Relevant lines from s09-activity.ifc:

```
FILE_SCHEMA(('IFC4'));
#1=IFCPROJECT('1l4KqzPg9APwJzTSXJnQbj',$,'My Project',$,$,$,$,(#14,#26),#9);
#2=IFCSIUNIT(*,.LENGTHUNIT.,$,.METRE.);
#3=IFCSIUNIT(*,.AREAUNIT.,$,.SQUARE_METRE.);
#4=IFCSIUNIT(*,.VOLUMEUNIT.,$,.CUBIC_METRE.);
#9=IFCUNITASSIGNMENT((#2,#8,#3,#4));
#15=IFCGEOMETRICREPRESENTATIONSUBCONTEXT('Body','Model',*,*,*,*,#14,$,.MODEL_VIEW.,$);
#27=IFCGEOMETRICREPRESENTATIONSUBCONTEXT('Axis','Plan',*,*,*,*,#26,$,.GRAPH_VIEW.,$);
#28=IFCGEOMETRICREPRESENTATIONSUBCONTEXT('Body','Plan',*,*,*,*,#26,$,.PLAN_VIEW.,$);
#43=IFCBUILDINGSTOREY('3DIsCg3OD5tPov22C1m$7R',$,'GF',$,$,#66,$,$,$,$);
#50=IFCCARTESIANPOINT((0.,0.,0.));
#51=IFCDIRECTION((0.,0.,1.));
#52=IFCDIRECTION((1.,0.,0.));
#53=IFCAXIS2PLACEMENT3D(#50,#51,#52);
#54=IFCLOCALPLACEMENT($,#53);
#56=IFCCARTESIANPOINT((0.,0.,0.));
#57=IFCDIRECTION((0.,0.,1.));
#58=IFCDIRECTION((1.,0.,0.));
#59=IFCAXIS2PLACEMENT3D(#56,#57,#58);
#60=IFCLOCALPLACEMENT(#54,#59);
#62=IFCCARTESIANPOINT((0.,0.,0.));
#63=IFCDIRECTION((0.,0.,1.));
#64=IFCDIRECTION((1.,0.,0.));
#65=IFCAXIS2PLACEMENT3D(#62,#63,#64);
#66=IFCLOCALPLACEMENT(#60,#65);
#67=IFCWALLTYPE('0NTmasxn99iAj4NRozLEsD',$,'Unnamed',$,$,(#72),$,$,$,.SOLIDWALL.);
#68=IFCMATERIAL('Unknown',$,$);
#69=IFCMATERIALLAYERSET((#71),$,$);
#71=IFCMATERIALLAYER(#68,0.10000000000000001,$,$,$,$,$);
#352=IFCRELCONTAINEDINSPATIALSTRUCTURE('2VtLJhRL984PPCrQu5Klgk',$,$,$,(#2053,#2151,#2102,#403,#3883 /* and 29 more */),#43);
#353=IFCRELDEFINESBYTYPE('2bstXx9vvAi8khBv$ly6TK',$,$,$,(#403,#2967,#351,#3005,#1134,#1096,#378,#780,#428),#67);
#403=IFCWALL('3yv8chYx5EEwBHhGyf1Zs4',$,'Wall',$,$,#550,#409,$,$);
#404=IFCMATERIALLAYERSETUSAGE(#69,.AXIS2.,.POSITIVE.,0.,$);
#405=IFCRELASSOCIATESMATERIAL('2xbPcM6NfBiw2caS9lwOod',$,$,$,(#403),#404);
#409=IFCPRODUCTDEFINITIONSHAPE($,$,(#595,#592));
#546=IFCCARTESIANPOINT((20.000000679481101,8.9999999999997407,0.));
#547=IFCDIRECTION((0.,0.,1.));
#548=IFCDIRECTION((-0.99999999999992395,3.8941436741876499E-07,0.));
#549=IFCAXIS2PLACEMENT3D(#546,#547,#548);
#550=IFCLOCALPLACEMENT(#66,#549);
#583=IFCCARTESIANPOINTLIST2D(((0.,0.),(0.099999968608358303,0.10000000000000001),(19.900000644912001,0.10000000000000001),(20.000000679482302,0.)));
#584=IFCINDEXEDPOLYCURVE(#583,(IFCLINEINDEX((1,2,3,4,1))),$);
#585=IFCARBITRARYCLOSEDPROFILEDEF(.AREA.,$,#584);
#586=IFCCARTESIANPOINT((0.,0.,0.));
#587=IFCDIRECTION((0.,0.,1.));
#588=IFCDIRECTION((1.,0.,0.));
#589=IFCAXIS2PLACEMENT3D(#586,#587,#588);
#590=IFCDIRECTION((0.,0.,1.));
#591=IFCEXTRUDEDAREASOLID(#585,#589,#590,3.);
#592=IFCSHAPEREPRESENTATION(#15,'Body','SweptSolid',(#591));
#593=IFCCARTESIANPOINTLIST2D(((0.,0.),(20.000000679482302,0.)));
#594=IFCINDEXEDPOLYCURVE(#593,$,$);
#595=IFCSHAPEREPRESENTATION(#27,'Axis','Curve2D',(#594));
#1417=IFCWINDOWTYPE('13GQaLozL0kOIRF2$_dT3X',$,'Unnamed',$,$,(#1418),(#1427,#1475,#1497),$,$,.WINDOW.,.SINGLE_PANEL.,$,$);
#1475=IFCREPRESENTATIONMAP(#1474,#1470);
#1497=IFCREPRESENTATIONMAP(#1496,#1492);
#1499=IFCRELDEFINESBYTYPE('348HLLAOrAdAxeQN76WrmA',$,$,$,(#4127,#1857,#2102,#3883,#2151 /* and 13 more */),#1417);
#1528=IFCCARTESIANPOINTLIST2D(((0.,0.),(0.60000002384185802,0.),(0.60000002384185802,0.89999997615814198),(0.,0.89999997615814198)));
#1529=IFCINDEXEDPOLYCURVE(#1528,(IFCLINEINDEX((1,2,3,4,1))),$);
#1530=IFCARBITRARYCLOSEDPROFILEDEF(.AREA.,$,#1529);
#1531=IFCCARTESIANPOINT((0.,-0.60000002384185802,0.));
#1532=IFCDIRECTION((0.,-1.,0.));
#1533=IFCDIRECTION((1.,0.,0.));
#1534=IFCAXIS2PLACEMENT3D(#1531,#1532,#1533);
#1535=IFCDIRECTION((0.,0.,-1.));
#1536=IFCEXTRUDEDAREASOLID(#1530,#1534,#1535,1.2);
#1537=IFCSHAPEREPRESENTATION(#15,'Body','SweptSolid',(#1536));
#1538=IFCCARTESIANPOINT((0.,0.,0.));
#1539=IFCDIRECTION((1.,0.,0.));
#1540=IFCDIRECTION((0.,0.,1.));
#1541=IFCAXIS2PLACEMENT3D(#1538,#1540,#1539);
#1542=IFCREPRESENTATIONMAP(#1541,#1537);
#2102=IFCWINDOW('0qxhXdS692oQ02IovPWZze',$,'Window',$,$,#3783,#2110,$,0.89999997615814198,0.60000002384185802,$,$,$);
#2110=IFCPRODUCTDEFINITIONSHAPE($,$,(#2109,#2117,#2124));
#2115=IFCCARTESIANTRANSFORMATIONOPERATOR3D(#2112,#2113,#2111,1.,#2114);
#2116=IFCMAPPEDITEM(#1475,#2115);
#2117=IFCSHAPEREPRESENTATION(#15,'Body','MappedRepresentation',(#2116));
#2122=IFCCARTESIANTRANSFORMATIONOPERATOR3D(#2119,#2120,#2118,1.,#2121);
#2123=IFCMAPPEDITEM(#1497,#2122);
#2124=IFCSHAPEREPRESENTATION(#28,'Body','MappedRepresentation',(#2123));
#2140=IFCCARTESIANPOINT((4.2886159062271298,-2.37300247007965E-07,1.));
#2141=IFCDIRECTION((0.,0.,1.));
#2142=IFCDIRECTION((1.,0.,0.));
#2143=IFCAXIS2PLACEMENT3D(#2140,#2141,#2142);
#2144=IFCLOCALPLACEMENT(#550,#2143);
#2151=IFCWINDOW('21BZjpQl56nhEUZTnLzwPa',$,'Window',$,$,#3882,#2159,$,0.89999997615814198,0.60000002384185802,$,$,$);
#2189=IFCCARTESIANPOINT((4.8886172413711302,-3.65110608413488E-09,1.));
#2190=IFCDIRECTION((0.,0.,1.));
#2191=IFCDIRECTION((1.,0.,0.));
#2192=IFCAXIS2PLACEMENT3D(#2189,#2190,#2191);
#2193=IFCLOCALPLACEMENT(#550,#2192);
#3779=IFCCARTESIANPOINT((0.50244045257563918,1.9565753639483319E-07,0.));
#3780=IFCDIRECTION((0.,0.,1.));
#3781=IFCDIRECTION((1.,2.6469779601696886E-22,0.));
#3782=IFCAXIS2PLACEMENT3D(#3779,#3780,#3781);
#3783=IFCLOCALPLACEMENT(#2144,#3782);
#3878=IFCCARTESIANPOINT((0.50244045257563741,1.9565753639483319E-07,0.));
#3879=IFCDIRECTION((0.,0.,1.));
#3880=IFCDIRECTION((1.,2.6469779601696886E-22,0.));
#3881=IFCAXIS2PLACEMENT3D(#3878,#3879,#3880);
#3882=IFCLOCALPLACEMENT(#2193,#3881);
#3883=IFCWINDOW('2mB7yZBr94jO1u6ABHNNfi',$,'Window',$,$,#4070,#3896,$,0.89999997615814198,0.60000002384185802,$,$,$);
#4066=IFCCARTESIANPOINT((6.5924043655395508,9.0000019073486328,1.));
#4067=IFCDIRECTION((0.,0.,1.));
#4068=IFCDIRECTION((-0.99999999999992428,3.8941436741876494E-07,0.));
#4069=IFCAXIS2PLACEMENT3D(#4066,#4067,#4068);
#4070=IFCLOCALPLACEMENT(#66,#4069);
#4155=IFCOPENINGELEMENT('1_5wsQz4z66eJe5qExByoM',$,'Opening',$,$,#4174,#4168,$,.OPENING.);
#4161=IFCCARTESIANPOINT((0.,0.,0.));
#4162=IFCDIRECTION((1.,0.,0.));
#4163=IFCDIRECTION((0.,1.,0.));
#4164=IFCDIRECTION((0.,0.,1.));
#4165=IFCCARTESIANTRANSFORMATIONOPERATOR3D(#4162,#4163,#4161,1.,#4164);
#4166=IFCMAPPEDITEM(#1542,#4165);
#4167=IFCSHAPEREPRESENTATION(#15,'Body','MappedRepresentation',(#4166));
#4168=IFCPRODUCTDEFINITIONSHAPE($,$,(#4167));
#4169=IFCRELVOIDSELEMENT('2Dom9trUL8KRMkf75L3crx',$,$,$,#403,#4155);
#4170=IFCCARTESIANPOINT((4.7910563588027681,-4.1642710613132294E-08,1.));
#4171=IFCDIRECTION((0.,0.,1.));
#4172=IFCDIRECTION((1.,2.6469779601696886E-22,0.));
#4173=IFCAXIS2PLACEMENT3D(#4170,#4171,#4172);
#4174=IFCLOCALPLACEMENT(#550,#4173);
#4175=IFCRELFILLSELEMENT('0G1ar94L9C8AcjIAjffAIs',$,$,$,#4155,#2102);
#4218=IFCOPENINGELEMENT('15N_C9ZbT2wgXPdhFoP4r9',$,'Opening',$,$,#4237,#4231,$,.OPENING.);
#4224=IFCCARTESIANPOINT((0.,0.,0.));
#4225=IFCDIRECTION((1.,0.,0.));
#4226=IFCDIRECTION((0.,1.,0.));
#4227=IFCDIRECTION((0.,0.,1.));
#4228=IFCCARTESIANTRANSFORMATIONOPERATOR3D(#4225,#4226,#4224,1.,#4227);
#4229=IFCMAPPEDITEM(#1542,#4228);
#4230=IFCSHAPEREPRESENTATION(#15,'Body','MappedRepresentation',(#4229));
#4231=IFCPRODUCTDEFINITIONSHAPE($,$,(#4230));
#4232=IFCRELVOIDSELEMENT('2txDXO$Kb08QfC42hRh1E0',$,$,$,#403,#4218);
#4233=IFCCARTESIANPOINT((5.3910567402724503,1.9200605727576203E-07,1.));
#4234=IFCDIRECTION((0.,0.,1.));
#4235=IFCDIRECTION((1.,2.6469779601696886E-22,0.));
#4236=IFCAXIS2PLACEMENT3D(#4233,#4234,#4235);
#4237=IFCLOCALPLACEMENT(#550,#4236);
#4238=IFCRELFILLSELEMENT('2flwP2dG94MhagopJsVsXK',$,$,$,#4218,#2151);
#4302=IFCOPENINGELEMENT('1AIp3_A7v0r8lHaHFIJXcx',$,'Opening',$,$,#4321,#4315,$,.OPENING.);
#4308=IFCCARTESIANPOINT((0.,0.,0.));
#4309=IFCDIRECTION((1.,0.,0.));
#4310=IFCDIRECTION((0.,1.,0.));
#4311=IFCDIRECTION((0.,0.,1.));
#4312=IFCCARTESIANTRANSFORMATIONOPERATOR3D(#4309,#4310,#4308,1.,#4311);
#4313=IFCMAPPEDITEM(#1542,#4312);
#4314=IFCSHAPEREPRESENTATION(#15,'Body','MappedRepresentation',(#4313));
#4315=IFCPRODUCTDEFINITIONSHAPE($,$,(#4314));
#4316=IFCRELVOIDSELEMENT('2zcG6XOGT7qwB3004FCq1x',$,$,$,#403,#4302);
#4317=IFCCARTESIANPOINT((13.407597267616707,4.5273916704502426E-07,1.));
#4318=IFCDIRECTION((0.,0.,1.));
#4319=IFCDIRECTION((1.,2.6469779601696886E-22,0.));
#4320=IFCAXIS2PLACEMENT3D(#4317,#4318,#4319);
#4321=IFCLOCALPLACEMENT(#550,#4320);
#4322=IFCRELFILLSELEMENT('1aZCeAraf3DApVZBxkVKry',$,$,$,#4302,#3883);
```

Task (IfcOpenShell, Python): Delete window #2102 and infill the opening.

```python
import ifcopenshell
import ifcopenshell.api.feature
import ifcopenshell.api.root
import ifcopenshell.geom
import ifcopenshell.util.shape

model = ifcopenshell.open("s09-activity.ifc")
settings = ifcopenshell.geom.settings()


def volume(element):
    """Net volume in cubic metres, openings subtracted."""
    shape = ifcopenshell.geom.create_shape(settings, element)
    return ifcopenshell.util.shape.get_volume(shape.geometry)


window = model.by_guid("0qxhXdS692oQ02IovPWZze")
opening = window.FillsVoids[0].RelatingOpeningElement
wall = opening.VoidsElements[0].RelatingBuildingElement
before = volume(wall)

ifcopenshell.api.root.remove_product(model, product=window)
ifcopenshell.api.feature.remove_feature(model, feature=opening)

after = volume(wall)

print(f"wall volume {before:.3f} -> {after:.3f} m3")

model.write("s09-activity_v2.ifc")
```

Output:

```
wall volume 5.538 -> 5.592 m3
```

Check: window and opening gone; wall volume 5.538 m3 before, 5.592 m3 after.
